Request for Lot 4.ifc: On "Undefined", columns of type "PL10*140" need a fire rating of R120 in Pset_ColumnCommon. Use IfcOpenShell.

First a look at what the model holds.

```python
import ifcopenshell
import ifcopenshell.util.element

model = ifcopenshell.open("Lot 4.ifc")
print(model.schema)
storey = next(s for s in model.by_type("IfcBuildingStorey") if s.Name == "Undefined")
columns = [e for e in ifcopenshell.util.element.get_decomposition(storey) if e.is_a("IfcColumn")]
seen = {}
for e in columns:
    element_type = ifcopenshell.util.element.get_type(e)
    key = (element_type.Name if element_type != e and element_type else None, ifcopenshell.util.element.get_pset(e, "Pset_ColumnCommon", "FireRating"))
    seen[key] = seen.get(key, 0) + 1
for (name, value), count in sorted(seen.items(), key=str):
    print(count, "x", name, "|", value)
```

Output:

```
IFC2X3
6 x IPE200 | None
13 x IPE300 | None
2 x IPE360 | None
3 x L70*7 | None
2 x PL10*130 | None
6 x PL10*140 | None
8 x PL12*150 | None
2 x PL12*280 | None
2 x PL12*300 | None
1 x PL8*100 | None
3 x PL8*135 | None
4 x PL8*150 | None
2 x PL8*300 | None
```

```python
import ifcopenshell
import ifcopenshell.api.pset
import ifcopenshell.util.element

model = ifcopenshell.open("Lot 4.ifc")

storey = next(s for s in model.by_type("IfcBuildingStorey") if s.Name == "Undefined")
columns = [e for e in ifcopenshell.util.element.get_decomposition(storey) if e.is_a("IfcColumn")]

count = 0
for e in columns:
    element_type = ifcopenshell.util.element.get_type(e)
    if element_type in (None, e) or element_type.Name != "PL10*140":
        continue
    found = ifcopenshell.util.element.get_pset(e, "Pset_ColumnCommon", should_inherit=False)
    if found:
        pset = model.by_id(found["id"])
        if len(ifcopenshell.util.element.get_elements_by_pset(pset)) > 1:
            pset = ifcopenshell.api.pset.unshare_pset(model, products=[e], pset=pset)[0]
    else:
        pset = ifcopenshell.api.pset.add_pset(model, product=e, name="Pset_ColumnCommon")
    ifcopenshell.api.pset.edit_pset(model, pset=pset, properties={"FireRating": "R120"})
    count += 1

print(count, "columns updated")

model.write("Lot 4-out.ifc")
```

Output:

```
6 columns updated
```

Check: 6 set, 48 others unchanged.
